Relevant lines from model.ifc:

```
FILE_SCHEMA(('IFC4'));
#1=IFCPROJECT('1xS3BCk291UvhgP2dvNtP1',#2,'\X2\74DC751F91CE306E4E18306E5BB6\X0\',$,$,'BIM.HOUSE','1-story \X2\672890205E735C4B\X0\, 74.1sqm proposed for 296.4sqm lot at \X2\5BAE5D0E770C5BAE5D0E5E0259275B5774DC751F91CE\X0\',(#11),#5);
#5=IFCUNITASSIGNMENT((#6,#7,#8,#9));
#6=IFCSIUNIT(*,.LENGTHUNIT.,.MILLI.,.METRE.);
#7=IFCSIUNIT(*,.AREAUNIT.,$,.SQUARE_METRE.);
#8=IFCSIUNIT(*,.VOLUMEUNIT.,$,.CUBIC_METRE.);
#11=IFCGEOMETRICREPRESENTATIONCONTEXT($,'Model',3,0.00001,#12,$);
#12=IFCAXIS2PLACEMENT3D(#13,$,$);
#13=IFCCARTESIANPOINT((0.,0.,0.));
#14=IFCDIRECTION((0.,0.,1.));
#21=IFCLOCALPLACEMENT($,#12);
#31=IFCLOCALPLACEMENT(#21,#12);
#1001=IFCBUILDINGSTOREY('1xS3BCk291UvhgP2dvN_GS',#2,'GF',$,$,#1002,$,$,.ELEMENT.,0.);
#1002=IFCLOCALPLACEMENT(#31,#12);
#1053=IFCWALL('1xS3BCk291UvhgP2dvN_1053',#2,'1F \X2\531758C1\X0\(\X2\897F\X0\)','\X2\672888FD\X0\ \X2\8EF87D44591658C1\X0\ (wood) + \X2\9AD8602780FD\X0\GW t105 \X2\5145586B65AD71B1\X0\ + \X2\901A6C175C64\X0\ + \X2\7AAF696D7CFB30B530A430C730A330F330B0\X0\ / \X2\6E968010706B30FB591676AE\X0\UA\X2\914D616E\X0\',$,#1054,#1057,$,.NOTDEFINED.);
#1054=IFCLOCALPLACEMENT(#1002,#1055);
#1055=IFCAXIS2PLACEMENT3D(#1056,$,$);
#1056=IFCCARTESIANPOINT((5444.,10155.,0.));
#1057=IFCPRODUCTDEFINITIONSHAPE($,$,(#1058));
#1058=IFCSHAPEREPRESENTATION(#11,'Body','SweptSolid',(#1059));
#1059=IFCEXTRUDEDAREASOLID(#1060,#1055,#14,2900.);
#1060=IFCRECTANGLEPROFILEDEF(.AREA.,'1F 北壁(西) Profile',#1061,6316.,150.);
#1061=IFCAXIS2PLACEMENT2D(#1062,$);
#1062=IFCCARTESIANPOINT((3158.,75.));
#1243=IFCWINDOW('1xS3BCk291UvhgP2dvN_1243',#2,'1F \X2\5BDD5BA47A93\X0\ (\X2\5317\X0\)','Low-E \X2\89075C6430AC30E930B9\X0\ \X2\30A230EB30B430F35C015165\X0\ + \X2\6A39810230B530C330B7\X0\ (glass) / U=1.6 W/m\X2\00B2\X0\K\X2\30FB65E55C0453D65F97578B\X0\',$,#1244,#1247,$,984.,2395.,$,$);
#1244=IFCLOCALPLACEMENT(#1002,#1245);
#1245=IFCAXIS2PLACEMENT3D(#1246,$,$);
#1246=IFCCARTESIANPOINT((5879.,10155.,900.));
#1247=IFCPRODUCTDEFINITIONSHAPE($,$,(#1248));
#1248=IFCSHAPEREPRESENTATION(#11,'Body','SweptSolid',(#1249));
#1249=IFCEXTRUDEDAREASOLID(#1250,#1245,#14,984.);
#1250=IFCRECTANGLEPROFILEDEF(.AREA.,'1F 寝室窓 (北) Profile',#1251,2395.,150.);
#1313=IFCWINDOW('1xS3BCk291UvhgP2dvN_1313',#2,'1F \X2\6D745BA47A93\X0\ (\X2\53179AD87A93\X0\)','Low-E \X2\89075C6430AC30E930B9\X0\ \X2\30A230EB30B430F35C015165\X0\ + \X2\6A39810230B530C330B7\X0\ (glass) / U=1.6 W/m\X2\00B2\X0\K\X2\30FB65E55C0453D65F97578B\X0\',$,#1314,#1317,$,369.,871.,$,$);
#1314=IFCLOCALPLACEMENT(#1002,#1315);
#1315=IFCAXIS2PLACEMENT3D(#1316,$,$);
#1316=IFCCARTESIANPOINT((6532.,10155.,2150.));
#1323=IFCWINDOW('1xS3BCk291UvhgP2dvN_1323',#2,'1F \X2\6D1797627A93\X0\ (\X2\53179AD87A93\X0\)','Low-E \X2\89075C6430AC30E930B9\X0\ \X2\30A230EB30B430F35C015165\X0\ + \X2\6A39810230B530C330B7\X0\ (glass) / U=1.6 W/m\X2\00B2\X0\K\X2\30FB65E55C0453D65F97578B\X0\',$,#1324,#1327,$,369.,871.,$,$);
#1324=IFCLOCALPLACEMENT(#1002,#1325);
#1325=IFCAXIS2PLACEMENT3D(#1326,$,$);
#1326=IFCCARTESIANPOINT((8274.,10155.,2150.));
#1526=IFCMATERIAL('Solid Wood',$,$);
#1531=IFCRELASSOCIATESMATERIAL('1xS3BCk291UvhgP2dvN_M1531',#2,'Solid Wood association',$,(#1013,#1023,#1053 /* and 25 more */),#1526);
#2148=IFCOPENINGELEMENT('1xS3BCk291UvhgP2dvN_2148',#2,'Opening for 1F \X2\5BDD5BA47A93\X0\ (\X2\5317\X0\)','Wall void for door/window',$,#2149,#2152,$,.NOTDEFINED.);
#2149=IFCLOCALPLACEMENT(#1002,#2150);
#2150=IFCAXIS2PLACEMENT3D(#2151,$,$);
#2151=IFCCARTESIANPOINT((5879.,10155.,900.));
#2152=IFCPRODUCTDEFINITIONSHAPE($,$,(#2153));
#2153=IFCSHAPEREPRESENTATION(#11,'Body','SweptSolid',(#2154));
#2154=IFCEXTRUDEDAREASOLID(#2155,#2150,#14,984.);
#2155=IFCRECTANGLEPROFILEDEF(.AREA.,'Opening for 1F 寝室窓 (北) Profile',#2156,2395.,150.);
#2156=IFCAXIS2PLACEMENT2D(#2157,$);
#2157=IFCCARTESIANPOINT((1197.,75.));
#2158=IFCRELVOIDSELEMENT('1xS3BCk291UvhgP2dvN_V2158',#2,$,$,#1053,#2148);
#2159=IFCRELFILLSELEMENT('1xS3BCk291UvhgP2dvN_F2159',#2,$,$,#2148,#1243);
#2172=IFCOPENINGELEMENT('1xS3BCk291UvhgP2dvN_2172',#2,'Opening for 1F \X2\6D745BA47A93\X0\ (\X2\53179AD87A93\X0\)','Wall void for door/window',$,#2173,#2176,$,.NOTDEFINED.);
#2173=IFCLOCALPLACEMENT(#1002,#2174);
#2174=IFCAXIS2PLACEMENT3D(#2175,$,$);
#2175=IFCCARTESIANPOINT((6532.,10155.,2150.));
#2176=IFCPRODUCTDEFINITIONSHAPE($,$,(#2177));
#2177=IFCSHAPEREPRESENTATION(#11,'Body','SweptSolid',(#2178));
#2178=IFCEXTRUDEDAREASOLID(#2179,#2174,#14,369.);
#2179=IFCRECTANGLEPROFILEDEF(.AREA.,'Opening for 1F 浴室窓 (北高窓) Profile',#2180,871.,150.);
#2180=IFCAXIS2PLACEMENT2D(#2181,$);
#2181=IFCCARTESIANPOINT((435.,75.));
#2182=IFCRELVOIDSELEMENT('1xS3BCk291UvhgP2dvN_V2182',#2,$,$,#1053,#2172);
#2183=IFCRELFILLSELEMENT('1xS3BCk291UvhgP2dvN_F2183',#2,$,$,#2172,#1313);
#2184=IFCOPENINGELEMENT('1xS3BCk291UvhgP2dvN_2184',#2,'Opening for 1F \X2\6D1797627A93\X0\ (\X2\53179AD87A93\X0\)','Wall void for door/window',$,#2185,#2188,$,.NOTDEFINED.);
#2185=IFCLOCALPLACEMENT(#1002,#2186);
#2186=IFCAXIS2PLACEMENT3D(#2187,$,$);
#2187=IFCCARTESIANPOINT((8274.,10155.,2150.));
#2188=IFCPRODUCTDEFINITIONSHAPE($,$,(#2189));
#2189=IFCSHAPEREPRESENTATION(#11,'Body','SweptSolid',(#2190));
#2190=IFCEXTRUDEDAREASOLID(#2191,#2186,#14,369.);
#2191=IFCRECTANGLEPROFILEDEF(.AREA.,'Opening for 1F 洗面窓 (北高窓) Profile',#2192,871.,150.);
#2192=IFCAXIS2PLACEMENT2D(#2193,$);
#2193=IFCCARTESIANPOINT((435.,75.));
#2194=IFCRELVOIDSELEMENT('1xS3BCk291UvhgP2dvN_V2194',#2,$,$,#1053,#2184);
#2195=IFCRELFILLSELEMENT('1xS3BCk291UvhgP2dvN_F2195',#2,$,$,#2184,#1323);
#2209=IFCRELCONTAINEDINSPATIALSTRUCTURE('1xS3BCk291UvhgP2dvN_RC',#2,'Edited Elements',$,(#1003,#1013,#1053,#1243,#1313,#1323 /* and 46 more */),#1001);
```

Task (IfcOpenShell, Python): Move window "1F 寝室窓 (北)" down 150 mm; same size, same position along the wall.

```python
import numpy as np
import ifcopenshell
import ifcopenshell.api.geometry
import ifcopenshell.util.placement
import ifcopenshell.util.unit

model = ifcopenshell.open("model.ifc")
unit_scale = ifcopenshell.util.unit.calculate_unit_scale(model)

window = model.by_guid("1xS3BCk291UvhgP2dvN_1243")
opening = window.FillsVoids[0].RelatingOpeningElement
dz = -150.0

shift = np.array([0.0, 0.0, dz])
# The window is not placed relative to its opening, so move both.
for product in (opening, window):
    matrix = ifcopenshell.util.placement.get_local_placement(product.ObjectPlacement)
    matrix[:3, 3] += shift
    ifcopenshell.api.geometry.edit_object_placement(model, product=product, matrix=matrix, is_si=False)

print(f"moved by {dz * unit_scale:+.3f} m")

model.write("model_v2.ifc")
```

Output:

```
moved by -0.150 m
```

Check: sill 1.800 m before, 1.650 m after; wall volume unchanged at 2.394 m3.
